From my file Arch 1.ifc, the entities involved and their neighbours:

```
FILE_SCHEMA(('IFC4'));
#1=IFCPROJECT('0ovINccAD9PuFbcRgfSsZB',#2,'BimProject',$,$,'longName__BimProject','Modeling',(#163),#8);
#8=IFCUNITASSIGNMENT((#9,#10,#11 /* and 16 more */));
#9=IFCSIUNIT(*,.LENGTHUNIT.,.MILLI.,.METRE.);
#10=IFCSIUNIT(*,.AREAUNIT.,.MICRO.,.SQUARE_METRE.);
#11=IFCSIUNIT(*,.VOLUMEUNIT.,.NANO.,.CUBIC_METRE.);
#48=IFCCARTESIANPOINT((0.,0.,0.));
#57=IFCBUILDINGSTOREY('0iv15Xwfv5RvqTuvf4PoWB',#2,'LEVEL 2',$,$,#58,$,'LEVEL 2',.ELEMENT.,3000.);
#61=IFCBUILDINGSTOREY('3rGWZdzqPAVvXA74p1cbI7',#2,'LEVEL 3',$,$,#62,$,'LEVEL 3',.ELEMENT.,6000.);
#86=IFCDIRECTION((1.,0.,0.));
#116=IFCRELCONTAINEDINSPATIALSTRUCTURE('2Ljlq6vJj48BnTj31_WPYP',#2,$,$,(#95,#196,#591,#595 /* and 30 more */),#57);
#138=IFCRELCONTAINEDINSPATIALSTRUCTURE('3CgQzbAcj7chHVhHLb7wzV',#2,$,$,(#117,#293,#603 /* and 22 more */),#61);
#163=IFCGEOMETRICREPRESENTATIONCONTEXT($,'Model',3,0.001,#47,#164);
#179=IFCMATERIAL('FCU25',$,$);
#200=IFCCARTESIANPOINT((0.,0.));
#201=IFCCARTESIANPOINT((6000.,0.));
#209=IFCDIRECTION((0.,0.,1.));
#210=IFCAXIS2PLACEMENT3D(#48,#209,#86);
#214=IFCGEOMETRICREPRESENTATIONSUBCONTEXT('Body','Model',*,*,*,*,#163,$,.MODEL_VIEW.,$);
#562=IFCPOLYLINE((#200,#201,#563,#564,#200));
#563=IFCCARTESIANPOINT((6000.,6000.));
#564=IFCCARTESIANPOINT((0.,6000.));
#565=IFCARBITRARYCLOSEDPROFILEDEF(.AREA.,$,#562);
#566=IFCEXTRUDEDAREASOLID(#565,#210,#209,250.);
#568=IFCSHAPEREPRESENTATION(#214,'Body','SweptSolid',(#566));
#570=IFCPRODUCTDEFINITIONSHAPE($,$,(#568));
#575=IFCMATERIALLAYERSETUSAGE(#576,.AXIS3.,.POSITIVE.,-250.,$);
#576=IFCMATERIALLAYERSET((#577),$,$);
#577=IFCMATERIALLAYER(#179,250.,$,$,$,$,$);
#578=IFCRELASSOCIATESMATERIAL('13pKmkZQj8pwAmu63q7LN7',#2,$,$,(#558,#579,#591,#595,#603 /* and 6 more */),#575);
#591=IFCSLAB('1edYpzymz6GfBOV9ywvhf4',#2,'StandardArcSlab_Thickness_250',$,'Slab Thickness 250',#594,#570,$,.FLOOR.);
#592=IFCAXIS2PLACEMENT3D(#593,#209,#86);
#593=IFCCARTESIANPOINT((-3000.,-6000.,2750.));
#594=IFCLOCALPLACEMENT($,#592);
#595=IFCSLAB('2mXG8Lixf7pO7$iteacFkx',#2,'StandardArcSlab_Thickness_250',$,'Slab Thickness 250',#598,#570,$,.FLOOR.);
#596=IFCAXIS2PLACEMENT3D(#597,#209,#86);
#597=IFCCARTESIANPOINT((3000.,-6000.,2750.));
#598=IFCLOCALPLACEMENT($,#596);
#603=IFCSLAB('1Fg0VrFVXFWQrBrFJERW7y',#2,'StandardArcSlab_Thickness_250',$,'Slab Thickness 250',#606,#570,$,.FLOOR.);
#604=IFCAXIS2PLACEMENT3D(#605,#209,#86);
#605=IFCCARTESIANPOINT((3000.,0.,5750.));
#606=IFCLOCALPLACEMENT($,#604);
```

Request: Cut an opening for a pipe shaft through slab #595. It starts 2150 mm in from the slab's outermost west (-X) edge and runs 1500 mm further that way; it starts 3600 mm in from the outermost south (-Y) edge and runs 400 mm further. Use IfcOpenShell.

```python
import numpy as np
import ifcopenshell
import ifcopenshell.api.feature
import ifcopenshell.api.geometry
import ifcopenshell.api.root
import ifcopenshell.geom
import ifcopenshell.util.placement
import ifcopenshell.util.representation
import ifcopenshell.util.shape
import ifcopenshell.util.unit

model = ifcopenshell.open("my file Arch 1.ifc")
unit_scale = ifcopenshell.util.unit.calculate_unit_scale(model)
settings = ifcopenshell.geom.settings()


def volume(element):
    """Net volume in cubic metres, openings subtracted."""
    shape = ifcopenshell.geom.create_shape(settings, element)
    return ifcopenshell.util.shape.get_volume(shape.geometry)


slab = model.by_id(595)
before = volume(slab)

# Extent in the slab's own axes, in metres. The edges named are its -X and -Y sides.
slab_shape = ifcopenshell.geom.create_shape(settings, slab)
vertices = ifcopenshell.util.shape.get_vertices(slab_shape.geometry)
x_min, y_min, bottom = vertices.min(axis=0)
top = vertices[:, 2].max()

opening = ifcopenshell.api.root.create_entity(model, ifc_class="IfcOpeningElement", name="Pipe shaft opening", predefined_type="OPENING")
context = ifcopenshell.util.representation.get_context(model, "Model", "Body", "MODEL_VIEW")
width, depth = 1.5, 0.4
outline = [(0.0, 0.0), (width, 0.0), (width, depth), (0.0, depth), (0.0, 0.0)]
# Overshoot both faces by 50 mm so the cut is clean.
shape = ifcopenshell.api.geometry.add_slab_representation(
    model, context=context, depth=top - bottom + 0.1, polyline=outline
)
ifcopenshell.api.geometry.assign_representation(model, product=opening, representation=shape)

matrix = ifcopenshell.util.placement.get_local_placement(slab.ObjectPlacement)
matrix[:, 3] = matrix @ np.append(np.array([x_min + 2.15, y_min + 3.6, bottom - 0.05]) / unit_scale, 1.0)
ifcopenshell.api.geometry.edit_object_placement(model, product=opening, matrix=matrix, is_si=False)
ifcopenshell.api.feature.add_feature(model, feature=opening, element=slab)

after = volume(slab)

print(f"slab volume {before:.3f} -> {after:.3f} m3")

model.write("my file Arch 1_updated.ifc")
```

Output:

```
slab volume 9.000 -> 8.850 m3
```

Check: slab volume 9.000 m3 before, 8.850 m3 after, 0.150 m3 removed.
